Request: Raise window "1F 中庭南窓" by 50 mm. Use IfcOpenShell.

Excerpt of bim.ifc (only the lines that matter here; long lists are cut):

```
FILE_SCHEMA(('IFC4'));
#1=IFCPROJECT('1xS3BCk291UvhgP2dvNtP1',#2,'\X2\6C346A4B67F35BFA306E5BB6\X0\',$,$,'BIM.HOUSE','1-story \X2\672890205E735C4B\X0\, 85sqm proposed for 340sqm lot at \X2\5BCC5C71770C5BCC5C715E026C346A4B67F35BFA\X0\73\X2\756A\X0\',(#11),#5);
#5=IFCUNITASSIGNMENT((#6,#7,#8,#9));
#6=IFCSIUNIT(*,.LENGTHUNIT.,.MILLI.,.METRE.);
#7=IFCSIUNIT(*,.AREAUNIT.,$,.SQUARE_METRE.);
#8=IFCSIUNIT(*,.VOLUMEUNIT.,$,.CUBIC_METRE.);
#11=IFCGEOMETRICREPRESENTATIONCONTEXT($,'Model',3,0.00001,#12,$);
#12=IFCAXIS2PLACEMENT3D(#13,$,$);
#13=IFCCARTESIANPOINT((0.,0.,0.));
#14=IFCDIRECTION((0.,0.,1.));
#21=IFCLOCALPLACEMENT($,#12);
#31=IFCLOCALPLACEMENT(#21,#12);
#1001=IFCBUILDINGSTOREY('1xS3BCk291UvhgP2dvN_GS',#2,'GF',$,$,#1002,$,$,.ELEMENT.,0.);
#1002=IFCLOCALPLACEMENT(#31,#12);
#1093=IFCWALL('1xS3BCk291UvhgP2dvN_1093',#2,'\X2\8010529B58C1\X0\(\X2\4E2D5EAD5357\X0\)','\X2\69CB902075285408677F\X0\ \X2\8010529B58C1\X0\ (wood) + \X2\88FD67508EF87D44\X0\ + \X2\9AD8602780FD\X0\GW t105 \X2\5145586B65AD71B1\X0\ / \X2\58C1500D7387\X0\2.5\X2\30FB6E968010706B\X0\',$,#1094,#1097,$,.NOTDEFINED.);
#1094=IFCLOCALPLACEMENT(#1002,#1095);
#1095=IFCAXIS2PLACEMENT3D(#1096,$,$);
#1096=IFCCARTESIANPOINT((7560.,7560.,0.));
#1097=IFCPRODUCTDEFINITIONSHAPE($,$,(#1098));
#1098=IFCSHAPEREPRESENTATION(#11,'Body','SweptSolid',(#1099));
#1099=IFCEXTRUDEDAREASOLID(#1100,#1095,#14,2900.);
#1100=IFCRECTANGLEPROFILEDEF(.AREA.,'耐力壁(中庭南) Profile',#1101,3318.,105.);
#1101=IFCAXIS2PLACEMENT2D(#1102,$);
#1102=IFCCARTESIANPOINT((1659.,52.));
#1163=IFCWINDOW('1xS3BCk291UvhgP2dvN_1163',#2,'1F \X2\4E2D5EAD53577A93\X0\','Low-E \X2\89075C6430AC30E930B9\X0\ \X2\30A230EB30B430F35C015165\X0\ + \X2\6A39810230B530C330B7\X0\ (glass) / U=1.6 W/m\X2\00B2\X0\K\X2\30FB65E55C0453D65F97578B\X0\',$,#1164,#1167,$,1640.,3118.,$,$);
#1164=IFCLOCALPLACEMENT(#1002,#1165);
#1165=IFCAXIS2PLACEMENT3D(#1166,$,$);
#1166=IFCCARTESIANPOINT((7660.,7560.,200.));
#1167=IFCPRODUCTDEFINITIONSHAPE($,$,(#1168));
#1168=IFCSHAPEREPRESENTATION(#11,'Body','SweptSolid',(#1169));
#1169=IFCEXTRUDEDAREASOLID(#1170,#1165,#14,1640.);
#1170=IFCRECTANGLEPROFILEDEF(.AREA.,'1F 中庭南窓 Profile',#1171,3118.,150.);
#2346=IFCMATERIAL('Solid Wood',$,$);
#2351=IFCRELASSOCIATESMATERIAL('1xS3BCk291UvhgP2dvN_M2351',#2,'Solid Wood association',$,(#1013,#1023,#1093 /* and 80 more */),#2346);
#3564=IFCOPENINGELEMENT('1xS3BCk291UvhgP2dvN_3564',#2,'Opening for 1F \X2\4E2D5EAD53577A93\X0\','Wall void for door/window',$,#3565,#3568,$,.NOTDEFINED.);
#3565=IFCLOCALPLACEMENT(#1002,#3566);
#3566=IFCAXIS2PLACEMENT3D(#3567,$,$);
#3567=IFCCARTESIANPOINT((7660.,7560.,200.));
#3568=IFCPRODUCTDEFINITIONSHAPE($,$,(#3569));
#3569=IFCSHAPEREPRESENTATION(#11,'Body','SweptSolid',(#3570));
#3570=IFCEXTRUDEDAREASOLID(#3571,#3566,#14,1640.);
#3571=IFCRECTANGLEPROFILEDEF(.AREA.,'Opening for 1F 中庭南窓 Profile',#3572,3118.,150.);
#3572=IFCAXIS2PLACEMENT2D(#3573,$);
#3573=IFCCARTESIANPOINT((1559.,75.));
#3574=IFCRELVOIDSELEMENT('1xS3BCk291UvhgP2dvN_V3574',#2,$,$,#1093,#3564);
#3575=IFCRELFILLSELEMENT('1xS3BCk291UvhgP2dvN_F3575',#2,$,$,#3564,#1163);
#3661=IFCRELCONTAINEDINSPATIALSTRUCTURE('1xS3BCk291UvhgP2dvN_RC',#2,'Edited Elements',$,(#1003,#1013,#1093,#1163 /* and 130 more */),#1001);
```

```python
import numpy as np
import ifcopenshell
import ifcopenshell.api.geometry
import ifcopenshell.util.placement
import ifcopenshell.util.unit

model = ifcopenshell.open("bim.ifc")
unit_scale = ifcopenshell.util.unit.calculate_unit_scale(model)

window = model.by_id(1163)
opening = window.FillsVoids[0].RelatingOpeningElement
dz = 50.0

shift = np.array([0.0, 0.0, dz])
# The window is not placed relative to its opening, so move both.
for product in (opening, window):
    matrix = ifcopenshell.util.placement.get_local_placement(product.ObjectPlacement)
    matrix[:3, 3] += shift
    ifcopenshell.api.geometry.edit_object_placement(model, product=product, matrix=matrix, is_si=False)

print(f"moved by {dz * unit_scale:+.3f} m")

model.write("bim_rev.ifc")
```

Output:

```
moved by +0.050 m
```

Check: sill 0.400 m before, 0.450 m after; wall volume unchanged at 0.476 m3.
